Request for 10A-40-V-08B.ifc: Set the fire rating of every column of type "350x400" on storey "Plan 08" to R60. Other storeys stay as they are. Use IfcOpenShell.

First a look at what the model holds.

```python
import ifcopenshell
import ifcopenshell.util.element

model = ifcopenshell.open("10A-40-V-08B.ifc")
print(model.schema)
storey = next(s for s in model.by_type("IfcBuildingStorey") if s.Name == "Plan 08")
columns = [e for e in ifcopenshell.util.element.get_decomposition(storey) if e.is_a("IfcColumn")]
seen = {}
for e in columns:
    element_type = ifcopenshell.util.element.get_type(e)
    key = (element_type.Name if element_type != e and element_type else None, ifcopenshell.util.element.get_pset(e, "Pset_ColumnCommon", "FireRating"))
    seen[key] = seen.get(key, 0) + 1
for (name, value), count in sorted(seen.items(), key=str):
    print(count, "x", name, "|", value)
```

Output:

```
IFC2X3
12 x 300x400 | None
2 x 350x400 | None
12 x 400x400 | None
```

```python
import ifcopenshell
import ifcopenshell.api.pset
import ifcopenshell.util.element

model = ifcopenshell.open("10A-40-V-08B.ifc")

storey = next(s for s in model.by_type("IfcBuildingStorey") if s.Name == "Plan 08")
columns = [e for e in ifcopenshell.util.element.get_decomposition(storey) if e.is_a("IfcColumn")]

count = 0
for e in columns:
    element_type = ifcopenshell.util.element.get_type(e)
    if element_type in (None, e) or element_type.Name != "350x400":
        continue
    # add_pset returns the element's existing set when there is one.
    pset = ifcopenshell.api.pset.add_pset(model, product=e, name="Pset_ColumnCommon")
    ifcopenshell.api.pset.edit_pset(model, pset=pset, properties={"FireRating": "R60"})
    count += 1

print(count, "columns updated")

model.write("10A-40-V-08B_updated.ifc")
```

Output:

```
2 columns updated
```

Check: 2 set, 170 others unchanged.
